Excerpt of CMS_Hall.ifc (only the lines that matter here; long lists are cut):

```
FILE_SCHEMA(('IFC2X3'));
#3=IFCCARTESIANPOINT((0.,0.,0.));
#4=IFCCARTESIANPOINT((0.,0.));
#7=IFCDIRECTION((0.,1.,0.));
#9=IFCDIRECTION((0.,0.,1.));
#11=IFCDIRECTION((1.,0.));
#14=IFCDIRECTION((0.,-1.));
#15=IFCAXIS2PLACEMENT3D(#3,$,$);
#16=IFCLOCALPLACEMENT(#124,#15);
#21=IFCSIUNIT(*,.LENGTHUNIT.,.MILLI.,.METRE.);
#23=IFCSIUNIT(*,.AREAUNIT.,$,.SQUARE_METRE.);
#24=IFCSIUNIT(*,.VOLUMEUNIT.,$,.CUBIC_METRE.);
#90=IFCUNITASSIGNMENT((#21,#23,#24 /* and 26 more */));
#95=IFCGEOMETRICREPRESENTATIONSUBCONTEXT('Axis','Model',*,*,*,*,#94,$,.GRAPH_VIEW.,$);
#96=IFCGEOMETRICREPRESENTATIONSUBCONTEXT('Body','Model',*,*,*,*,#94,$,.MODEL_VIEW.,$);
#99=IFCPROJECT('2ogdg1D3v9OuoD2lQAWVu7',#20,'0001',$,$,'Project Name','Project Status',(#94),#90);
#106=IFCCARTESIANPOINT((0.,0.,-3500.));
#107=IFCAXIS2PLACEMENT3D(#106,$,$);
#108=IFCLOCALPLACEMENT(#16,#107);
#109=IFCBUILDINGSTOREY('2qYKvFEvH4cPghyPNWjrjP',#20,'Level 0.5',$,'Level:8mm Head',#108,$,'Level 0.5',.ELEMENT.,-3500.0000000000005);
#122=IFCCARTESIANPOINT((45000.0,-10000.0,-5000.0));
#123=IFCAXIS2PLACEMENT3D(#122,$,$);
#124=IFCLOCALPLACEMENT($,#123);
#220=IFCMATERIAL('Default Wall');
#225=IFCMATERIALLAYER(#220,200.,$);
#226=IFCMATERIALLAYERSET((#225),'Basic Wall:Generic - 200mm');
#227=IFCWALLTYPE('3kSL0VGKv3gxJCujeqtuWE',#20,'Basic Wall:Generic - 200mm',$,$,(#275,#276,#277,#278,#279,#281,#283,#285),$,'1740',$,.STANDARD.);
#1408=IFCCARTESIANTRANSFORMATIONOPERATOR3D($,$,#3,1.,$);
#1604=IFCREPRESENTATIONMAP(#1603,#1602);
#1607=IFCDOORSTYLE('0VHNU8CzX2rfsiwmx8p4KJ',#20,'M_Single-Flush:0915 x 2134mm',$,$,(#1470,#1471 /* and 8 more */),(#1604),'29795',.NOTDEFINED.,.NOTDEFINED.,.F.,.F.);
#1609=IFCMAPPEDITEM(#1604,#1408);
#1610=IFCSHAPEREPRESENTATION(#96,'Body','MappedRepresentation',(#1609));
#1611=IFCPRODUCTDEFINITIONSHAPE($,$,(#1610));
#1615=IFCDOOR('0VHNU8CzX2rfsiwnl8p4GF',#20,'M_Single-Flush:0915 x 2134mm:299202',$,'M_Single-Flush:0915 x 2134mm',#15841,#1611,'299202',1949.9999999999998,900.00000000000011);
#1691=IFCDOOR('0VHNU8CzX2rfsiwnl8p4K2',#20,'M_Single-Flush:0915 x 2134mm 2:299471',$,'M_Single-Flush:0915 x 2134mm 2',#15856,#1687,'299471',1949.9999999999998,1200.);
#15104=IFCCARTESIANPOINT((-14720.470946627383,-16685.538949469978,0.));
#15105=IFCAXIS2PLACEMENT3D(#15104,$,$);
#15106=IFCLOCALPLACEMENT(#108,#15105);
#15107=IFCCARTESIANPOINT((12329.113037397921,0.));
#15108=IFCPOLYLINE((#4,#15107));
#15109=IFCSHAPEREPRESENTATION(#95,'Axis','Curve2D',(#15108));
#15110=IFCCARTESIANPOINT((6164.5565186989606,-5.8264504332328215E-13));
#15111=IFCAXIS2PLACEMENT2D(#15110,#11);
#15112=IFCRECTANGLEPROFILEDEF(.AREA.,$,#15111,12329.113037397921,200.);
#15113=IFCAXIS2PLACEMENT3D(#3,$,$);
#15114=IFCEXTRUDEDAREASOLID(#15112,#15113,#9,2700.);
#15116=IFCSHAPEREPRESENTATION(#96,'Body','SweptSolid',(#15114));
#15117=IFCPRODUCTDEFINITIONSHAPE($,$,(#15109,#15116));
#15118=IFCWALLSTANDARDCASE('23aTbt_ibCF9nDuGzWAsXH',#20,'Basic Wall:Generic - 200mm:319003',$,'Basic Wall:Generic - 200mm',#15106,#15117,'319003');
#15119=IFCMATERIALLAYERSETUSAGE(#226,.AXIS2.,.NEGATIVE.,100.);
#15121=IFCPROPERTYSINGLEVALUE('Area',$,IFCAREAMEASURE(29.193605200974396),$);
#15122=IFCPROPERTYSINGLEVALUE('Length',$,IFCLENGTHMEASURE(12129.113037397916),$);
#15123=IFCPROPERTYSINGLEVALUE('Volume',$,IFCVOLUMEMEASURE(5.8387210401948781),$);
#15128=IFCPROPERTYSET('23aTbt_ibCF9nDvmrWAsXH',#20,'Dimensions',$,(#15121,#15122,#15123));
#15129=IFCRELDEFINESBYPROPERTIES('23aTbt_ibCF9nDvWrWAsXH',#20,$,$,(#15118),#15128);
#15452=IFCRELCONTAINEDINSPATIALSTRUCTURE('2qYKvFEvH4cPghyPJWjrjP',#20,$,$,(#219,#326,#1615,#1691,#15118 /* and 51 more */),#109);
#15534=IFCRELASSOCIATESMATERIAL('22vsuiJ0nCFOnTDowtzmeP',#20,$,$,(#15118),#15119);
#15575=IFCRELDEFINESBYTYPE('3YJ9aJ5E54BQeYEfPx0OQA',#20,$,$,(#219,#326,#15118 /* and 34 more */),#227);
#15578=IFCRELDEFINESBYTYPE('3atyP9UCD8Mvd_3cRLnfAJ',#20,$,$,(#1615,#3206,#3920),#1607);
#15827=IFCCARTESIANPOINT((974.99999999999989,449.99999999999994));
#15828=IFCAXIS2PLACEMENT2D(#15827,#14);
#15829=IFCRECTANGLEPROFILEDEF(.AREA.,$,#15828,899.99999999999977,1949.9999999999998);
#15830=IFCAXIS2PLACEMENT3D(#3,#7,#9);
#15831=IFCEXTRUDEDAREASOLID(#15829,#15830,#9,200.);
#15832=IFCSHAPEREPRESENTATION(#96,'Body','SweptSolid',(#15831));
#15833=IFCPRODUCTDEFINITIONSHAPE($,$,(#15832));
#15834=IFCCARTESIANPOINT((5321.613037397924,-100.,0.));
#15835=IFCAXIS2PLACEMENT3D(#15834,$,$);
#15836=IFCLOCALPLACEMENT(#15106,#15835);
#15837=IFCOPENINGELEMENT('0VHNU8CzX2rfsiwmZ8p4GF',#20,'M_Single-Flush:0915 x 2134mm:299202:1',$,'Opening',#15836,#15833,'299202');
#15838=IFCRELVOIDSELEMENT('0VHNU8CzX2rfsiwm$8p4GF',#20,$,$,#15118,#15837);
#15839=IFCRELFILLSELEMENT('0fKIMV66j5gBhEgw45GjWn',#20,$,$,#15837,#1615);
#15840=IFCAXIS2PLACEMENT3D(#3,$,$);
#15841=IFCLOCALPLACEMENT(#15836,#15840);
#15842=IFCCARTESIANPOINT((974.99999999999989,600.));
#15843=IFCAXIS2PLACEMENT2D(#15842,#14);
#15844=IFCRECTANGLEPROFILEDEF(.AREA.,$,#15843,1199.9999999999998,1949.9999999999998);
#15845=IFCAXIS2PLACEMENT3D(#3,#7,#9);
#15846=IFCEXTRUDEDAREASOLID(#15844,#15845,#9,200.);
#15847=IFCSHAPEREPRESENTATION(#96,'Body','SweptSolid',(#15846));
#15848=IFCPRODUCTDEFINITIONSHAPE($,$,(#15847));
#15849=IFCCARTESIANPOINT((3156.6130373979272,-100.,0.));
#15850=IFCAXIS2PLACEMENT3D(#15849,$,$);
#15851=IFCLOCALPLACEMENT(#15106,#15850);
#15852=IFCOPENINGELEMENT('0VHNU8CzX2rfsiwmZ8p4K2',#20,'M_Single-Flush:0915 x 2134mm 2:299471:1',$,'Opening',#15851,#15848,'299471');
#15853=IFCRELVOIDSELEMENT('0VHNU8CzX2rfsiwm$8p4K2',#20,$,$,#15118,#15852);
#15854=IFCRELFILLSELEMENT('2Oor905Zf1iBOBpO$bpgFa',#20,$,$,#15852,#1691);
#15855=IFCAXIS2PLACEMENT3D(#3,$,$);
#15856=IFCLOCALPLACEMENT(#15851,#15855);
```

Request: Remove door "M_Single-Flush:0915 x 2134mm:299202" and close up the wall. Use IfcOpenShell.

```python
import ifcopenshell
import ifcopenshell.api.feature
import ifcopenshell.api.pset
import ifcopenshell.api.root
import ifcopenshell.geom
import ifcopenshell.util.element
import ifcopenshell.util.shape
import ifcopenshell.util.unit

model = ifcopenshell.open("CMS_Hall.ifc")
area_scale = ifcopenshell.util.unit.calculate_unit_scale(model, "AREAUNIT")
volume_scale = ifcopenshell.util.unit.calculate_unit_scale(model, "VOLUMEUNIT")
settings = ifcopenshell.geom.settings()


def volume(element):
    """Net volume in cubic metres, openings subtracted."""
    shape = ifcopenshell.geom.create_shape(settings, element)
    return ifcopenshell.util.shape.get_volume(shape.geometry)


door = model.by_guid("0VHNU8CzX2rfsiwnl8p4GF")
opening = door.FillsVoids[0].RelatingOpeningElement
wall = opening.VoidsElements[0].RelatingBuildingElement
before = volume(wall)

ifcopenshell.api.root.remove_product(model, product=door)
ifcopenshell.api.feature.remove_feature(model, feature=opening)

after = volume(wall)
thickness = 0.2  # wall thickness in metres

# Update the wall's stored quantities.
pset = model.by_id(ifcopenshell.util.element.get_pset(wall, "Dimensions", should_inherit=False)["id"])
ifcopenshell.api.pset.edit_pset(model, pset=pset, properties={
    "Area": model.create_entity("IfcAreaMeasure", after / thickness / area_scale),
    "Volume": model.create_entity("IfcVolumeMeasure", after / volume_scale),
})

print(f"wall volume {before:.3f} -> {after:.3f} m3")

model.write("CMS_Hall_v2.ifc")
```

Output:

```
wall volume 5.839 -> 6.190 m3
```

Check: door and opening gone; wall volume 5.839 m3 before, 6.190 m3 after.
